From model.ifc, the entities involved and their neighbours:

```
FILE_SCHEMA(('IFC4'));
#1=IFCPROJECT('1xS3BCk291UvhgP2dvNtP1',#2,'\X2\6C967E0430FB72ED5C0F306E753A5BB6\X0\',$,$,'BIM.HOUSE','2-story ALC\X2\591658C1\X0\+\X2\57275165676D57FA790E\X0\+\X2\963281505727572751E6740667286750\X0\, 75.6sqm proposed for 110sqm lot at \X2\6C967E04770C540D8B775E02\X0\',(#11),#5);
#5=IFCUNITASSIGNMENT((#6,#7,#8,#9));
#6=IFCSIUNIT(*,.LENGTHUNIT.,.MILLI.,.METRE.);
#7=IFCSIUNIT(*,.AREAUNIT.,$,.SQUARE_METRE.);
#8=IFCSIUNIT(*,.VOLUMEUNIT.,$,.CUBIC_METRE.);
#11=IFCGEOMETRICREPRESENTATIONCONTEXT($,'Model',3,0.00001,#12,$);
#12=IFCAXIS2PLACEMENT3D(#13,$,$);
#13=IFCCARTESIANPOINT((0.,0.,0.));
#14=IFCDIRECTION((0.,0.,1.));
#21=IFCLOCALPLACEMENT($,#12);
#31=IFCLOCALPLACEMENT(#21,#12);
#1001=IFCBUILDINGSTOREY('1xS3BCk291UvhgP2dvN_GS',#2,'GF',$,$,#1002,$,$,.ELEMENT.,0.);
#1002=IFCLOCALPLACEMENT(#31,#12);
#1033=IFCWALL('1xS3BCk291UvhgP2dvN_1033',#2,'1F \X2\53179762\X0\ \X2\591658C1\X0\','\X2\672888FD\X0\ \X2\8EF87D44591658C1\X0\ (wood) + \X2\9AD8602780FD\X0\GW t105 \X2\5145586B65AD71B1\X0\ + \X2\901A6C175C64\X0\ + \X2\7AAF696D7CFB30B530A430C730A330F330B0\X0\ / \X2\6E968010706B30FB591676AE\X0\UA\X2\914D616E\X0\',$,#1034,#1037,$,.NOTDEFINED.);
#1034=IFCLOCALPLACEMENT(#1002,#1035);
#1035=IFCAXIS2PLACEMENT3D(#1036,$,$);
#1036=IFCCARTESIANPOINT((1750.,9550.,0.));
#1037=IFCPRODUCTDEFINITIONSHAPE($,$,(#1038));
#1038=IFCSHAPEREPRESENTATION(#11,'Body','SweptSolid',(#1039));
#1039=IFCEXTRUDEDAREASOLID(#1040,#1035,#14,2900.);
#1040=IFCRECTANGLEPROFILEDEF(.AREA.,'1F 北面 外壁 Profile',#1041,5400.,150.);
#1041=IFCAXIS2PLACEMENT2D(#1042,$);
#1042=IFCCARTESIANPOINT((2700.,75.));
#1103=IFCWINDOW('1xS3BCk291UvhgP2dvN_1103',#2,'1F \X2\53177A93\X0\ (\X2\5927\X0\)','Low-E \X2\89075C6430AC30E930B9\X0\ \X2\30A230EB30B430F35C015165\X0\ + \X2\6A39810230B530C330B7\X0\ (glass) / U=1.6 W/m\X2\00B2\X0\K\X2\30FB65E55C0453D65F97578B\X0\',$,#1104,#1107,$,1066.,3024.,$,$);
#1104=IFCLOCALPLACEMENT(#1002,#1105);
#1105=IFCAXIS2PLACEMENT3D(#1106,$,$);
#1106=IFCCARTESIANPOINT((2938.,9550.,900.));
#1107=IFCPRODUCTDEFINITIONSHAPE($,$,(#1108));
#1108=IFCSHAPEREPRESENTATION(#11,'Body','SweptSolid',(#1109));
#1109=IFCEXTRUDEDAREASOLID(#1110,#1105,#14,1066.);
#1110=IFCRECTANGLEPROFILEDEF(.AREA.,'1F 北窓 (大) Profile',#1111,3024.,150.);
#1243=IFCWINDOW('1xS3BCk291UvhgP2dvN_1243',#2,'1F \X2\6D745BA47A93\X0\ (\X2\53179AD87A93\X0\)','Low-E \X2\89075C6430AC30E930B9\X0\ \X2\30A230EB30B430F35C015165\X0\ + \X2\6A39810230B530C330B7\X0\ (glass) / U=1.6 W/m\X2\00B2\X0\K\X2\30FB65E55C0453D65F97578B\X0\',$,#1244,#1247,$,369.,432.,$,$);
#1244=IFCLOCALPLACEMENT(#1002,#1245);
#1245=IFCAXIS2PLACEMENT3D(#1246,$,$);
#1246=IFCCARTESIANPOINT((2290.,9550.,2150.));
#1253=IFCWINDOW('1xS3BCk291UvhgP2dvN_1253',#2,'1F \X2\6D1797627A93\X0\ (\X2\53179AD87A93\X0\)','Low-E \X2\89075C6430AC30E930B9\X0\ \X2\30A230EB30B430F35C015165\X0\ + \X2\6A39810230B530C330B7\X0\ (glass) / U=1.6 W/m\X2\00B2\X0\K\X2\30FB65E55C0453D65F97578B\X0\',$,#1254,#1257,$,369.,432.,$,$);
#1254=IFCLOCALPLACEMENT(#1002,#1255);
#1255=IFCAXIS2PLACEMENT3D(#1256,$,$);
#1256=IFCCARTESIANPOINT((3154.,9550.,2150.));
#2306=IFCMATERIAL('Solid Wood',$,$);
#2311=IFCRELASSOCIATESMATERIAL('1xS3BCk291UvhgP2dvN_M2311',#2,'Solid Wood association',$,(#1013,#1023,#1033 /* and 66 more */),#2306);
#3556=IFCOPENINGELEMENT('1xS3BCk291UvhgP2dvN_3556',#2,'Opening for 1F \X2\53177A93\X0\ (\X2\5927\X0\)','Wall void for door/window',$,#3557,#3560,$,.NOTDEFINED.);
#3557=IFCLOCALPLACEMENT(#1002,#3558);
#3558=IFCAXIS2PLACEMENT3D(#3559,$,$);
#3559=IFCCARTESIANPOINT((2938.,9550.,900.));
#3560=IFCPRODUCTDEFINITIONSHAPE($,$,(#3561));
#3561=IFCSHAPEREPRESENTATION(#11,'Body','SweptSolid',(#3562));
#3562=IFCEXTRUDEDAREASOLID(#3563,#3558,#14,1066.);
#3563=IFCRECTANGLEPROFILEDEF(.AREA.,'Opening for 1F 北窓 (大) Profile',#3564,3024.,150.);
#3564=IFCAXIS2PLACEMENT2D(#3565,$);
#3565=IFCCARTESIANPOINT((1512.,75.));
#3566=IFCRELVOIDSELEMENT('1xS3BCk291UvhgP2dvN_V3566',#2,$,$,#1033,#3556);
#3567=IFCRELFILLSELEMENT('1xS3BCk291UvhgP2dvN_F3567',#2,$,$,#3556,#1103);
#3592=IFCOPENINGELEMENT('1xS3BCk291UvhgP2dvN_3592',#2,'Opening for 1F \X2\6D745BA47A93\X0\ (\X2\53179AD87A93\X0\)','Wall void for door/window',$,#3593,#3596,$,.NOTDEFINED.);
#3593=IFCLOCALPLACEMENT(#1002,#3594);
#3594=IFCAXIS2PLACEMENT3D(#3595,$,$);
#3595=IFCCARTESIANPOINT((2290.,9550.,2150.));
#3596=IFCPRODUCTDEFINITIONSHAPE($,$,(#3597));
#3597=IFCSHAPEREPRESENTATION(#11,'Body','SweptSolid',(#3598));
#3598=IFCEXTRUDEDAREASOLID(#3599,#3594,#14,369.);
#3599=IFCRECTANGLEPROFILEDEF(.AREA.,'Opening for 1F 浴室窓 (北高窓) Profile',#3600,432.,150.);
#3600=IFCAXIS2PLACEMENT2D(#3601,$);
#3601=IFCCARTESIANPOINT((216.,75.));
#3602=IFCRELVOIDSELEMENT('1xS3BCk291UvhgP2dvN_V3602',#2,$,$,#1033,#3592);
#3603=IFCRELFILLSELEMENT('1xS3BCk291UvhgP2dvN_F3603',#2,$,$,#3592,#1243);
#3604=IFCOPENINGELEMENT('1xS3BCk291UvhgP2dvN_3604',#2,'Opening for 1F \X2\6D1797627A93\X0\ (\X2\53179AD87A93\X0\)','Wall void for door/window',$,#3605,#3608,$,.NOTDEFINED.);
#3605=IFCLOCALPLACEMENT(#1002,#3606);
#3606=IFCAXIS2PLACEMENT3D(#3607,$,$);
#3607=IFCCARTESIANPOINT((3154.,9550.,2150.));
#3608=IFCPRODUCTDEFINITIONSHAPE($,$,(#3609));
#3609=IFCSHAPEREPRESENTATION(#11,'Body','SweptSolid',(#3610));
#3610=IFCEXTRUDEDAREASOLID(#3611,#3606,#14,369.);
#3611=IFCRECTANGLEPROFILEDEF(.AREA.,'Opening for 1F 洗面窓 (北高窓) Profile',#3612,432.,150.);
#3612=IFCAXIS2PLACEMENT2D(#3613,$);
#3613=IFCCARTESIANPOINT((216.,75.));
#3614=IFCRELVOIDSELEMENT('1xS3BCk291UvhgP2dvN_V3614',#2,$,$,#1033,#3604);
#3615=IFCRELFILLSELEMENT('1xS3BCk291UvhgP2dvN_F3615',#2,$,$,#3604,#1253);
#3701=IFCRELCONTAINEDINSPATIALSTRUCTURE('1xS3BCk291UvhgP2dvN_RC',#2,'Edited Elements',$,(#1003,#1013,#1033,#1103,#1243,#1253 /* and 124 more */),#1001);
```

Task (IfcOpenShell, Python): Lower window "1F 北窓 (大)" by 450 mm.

```python
import numpy as np
import ifcopenshell
import ifcopenshell.api.geometry
import ifcopenshell.util.placement
import ifcopenshell.util.unit

model = ifcopenshell.open("model.ifc")
unit_scale = ifcopenshell.util.unit.calculate_unit_scale(model)

window = model.by_id(1103)
opening = window.FillsVoids[0].RelatingOpeningElement
dz = -450.0

shift = np.array([0.0, 0.0, dz])
# The window is not placed relative to its opening, so move both.
for product in (opening, window):
    matrix = ifcopenshell.util.placement.get_local_placement(product.ObjectPlacement)
    matrix[:3, 3] += shift
    ifcopenshell.api.geometry.edit_object_placement(model, product=product, matrix=matrix, is_si=False)

print(f"moved by {dz * unit_scale:+.3f} m")

model.write("model-out.ifc")
```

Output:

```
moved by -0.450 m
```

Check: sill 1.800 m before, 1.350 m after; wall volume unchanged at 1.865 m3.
